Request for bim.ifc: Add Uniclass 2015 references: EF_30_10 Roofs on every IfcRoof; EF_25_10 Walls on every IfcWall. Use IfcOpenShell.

First a look at what the model holds.

```python
import ifcopenshell

model = ifcopenshell.open("bim.ifc")
print(model.schema)
print("classifications:", [c.Name for c in model.by_type("IfcClassification")])
for ifc_class in ("IfcDoor", "IfcRoof", "IfcStair", "IfcWall", "IfcWindow"):
    print(ifc_class, len(model.by_type(ifc_class)))
```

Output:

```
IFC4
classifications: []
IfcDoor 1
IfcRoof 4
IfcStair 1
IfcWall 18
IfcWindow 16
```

```python
import ifcopenshell
import ifcopenshell.api.classification

model = ifcopenshell.open("bim.ifc")

system = ifcopenshell.api.classification.add_classification(model, classification="Uniclass 2015")

codes = {
    "IfcRoof": ("EF_30_10", "Roofs"),
    "IfcWall": ("EF_25_10", "Walls"),
}
for ifc_class, (code, name) in codes.items():
    products = model.by_type(ifc_class)
    ifcopenshell.api.classification.add_reference(
        model, products=products, classification=system, identification=code, name=name
    )
    print(code, len(products))

model.write("bim_updated.ifc")
```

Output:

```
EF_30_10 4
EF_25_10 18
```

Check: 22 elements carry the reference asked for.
